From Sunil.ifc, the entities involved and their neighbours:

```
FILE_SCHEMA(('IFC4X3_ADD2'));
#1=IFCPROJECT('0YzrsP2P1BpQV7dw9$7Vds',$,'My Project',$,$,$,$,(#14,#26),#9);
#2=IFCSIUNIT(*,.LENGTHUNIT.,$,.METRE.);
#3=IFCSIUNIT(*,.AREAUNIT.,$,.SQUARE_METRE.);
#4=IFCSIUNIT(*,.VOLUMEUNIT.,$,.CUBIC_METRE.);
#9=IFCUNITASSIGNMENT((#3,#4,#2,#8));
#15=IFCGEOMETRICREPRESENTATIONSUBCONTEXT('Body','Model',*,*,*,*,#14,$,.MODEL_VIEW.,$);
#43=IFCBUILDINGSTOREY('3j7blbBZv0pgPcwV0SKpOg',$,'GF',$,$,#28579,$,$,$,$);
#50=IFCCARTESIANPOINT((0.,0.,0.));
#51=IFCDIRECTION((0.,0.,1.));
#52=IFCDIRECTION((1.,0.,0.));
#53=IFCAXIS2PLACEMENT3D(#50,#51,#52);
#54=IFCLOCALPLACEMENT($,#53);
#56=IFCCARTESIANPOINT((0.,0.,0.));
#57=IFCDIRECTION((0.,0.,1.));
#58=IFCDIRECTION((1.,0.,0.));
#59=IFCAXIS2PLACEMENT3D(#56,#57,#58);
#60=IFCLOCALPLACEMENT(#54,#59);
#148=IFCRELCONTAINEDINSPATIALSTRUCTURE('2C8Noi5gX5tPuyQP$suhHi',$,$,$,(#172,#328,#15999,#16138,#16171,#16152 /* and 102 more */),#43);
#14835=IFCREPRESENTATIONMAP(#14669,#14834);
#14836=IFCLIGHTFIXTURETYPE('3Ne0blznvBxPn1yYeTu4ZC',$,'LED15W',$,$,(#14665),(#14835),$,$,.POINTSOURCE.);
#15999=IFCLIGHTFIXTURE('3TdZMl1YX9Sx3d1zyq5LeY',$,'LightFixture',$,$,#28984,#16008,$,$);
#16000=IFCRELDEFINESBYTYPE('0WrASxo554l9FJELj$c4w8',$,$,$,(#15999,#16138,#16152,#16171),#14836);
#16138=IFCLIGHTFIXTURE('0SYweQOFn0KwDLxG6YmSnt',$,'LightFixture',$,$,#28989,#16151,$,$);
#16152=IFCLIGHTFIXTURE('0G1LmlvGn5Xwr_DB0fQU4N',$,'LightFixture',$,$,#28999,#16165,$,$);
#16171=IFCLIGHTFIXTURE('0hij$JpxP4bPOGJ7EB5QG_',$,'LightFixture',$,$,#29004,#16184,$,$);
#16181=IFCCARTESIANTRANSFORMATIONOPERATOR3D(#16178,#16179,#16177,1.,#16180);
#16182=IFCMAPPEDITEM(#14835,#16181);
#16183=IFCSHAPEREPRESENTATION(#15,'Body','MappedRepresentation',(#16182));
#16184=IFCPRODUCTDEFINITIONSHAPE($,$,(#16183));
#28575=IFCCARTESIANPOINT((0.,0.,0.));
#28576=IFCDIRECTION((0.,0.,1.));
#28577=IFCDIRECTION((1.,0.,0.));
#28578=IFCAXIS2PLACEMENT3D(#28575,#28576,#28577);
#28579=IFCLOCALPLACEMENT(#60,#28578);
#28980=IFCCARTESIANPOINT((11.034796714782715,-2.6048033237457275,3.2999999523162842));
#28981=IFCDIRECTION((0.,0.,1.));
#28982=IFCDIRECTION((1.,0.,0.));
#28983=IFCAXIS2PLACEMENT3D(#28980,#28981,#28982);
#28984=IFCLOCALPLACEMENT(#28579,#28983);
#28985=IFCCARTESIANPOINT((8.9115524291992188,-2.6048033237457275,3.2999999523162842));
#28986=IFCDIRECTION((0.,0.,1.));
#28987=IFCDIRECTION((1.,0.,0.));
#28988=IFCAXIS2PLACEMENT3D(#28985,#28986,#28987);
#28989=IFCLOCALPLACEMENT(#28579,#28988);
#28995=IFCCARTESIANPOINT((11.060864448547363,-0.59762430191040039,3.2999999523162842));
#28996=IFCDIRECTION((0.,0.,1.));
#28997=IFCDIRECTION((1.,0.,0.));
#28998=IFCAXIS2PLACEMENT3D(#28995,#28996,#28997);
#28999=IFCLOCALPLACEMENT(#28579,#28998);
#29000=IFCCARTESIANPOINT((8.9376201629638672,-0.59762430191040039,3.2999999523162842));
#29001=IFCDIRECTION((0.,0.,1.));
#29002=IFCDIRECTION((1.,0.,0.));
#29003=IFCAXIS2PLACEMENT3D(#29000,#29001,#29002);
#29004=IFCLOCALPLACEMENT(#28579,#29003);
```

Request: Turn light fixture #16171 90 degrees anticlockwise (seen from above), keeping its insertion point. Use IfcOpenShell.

```python
import ifcopenshell
import ifcopenshell.api.geometry
import ifcopenshell.util.placement

model = ifcopenshell.open("Sunil.ifc")

item = model.by_id(16171)
matrix = ifcopenshell.util.placement.get_local_placement(item.ObjectPlacement)
matrix = matrix @ ifcopenshell.util.placement.rotation(90, "Z")
ifcopenshell.api.geometry.edit_object_placement(model, product=item, matrix=matrix, is_si=False)

print(ifcopenshell.util.placement.get_local_placement(item.ObjectPlacement).round(3) + 0.0)

model.write("Sunil_v2.ifc")
```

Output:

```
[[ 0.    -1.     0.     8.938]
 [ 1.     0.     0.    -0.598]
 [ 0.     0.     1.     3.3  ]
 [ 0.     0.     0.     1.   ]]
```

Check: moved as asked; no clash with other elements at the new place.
